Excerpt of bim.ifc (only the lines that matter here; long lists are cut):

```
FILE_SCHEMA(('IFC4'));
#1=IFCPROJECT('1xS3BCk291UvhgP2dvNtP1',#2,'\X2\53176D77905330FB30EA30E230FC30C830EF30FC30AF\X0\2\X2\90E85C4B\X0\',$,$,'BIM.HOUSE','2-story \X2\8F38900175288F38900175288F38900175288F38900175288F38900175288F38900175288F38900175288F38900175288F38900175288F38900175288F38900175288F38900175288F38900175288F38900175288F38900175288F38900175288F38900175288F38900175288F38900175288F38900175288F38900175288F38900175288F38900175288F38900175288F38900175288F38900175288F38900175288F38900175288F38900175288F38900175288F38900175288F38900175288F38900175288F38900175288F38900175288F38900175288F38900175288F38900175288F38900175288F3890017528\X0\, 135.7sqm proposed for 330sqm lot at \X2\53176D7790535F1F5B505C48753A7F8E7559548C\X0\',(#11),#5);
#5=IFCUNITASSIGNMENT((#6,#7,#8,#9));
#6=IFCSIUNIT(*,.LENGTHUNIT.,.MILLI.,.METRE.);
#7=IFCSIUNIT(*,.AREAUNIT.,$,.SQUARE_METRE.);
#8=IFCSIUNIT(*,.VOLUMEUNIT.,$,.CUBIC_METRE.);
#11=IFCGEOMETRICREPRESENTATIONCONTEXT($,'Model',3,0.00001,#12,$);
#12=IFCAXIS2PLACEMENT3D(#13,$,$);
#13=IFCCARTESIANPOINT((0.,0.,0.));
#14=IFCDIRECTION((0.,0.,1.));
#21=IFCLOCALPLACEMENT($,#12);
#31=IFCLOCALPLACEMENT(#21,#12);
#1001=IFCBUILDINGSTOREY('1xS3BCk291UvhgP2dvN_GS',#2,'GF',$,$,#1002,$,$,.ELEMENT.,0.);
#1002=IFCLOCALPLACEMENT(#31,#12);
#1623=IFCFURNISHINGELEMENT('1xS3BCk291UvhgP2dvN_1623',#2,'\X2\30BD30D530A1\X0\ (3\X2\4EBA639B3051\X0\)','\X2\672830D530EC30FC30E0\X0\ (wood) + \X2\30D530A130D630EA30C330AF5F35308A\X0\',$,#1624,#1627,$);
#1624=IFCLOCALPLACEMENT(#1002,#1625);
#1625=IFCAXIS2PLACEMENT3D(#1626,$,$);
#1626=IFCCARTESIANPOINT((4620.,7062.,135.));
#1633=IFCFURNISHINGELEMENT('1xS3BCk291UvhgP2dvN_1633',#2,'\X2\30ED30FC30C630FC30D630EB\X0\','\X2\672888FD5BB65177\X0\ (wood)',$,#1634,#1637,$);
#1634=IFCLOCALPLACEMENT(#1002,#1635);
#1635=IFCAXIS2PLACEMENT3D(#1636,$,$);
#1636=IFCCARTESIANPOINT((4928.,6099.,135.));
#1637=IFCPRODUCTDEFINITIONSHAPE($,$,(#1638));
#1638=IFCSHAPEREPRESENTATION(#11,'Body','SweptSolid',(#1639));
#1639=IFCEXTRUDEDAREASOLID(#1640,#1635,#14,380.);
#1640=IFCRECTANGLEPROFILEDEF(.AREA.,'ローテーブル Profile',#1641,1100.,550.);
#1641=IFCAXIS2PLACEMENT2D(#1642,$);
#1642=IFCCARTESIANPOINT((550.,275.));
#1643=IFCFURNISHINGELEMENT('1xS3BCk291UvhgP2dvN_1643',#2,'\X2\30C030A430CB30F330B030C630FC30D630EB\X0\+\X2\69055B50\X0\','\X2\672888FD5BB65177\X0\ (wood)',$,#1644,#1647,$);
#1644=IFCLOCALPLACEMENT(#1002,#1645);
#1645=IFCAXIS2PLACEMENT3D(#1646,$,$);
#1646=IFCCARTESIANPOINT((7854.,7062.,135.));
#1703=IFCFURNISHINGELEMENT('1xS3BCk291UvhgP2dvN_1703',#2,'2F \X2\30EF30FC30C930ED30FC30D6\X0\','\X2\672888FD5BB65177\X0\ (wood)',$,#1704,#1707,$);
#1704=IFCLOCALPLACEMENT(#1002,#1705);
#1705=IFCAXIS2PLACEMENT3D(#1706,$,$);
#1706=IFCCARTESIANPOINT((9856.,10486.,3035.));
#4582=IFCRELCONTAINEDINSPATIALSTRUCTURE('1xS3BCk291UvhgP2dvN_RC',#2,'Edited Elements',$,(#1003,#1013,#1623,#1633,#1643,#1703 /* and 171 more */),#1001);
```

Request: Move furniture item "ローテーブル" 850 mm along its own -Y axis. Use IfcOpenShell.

```python
import ifcopenshell
import ifcopenshell.api.geometry
import ifcopenshell.util.placement
import ifcopenshell.util.unit

model = ifcopenshell.open("bim.ifc")
unit_scale = ifcopenshell.util.unit.calculate_unit_scale(model)

item = model.by_guid("1xS3BCk291UvhgP2dvN_1633")
matrix = ifcopenshell.util.placement.get_local_placement(item.ObjectPlacement)
matrix[:3, 3] -= matrix[:3, 1] * 0.85 / unit_scale
ifcopenshell.api.geometry.edit_object_placement(model, product=item, matrix=matrix, is_si=False)

print(ifcopenshell.util.placement.get_local_placement(item.ObjectPlacement).round(3) + 0.0)

model.write("bim_rev.ifc")
```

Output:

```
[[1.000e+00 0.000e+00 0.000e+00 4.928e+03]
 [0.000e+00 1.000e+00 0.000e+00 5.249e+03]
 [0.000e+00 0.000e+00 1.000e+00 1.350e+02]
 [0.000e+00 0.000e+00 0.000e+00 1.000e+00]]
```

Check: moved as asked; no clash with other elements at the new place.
